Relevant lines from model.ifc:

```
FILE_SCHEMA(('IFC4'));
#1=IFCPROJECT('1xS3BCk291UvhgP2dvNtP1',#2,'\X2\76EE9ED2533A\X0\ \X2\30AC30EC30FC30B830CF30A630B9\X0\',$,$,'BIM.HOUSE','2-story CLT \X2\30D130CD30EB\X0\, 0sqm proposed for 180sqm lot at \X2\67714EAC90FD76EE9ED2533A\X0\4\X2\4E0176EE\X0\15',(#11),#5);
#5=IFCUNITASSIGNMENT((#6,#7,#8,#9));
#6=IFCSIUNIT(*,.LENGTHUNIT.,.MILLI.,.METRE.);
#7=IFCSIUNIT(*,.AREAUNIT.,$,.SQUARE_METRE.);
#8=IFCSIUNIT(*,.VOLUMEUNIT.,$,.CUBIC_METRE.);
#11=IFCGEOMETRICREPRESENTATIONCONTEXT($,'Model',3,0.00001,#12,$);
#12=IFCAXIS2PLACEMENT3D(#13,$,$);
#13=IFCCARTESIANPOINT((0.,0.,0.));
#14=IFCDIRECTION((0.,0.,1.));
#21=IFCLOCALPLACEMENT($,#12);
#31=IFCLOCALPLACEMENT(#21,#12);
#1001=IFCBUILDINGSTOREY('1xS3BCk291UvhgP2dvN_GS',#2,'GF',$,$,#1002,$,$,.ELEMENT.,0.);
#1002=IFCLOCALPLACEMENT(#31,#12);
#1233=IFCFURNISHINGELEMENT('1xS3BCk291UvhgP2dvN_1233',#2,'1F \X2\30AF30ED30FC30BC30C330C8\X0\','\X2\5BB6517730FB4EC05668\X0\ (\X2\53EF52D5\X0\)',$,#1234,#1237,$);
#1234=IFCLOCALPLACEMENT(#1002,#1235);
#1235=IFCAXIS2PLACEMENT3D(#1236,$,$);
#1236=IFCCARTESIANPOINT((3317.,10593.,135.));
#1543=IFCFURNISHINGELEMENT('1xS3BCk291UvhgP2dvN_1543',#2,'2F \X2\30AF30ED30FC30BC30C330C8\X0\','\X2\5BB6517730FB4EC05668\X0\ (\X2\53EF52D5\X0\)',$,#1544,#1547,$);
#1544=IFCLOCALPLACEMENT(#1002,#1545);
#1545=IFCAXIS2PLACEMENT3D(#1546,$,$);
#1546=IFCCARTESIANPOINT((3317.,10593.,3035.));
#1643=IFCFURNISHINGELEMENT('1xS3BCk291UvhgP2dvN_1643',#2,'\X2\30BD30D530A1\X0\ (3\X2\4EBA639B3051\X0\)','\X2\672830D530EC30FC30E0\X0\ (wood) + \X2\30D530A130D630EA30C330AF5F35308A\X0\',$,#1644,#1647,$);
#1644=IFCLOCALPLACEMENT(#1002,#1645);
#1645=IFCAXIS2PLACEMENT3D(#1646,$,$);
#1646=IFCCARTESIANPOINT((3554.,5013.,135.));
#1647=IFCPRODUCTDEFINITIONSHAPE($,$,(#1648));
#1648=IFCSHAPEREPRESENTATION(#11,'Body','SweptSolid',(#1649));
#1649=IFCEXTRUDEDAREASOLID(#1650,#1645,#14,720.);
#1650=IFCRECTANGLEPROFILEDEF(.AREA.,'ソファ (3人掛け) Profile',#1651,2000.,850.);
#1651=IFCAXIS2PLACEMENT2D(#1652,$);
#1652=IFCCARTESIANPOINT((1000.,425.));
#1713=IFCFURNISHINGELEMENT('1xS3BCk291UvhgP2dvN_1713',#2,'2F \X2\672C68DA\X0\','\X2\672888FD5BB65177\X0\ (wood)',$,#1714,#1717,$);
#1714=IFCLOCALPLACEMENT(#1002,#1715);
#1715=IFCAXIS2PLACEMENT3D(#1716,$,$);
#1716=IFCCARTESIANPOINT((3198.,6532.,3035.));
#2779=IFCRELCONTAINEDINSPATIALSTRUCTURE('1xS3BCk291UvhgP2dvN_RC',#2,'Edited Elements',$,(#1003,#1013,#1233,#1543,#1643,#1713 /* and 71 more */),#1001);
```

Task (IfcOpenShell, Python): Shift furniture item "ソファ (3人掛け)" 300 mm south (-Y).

```python
import ifcopenshell
import ifcopenshell.api.geometry
import ifcopenshell.util.placement

model = ifcopenshell.open("model.ifc")

item = model.by_guid("1xS3BCk291UvhgP2dvN_1643")
matrix = ifcopenshell.util.placement.get_local_placement(item.ObjectPlacement)
matrix[1, 3] -= 300.0
ifcopenshell.api.geometry.edit_object_placement(model, product=item, matrix=matrix, is_si=False)

print(ifcopenshell.util.placement.get_local_placement(item.ObjectPlacement).round(3) + 0.0)

model.write("model-out.ifc")
```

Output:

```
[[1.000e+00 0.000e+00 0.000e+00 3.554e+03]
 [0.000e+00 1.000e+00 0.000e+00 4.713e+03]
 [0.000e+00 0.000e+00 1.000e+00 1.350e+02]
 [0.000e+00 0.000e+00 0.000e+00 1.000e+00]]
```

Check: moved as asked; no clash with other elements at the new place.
